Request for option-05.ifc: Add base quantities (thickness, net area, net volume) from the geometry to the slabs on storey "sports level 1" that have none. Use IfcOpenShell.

First a look at what the model holds.

```python
import ifcopenshell
import ifcopenshell.util.element
import ifcopenshell.util.unit

model = ifcopenshell.open("option-05.ifc")
print(model.schema)
for unit_type in ("LENGTHUNIT", "AREAUNIT", "VOLUMEUNIT"):
    print(unit_type, ifcopenshell.util.unit.calculate_unit_scale(model, unit_type))
storey = next(s for s in model.by_type("IfcBuildingStorey") if s.Name == "sports level 1")
slabs = [e for e in ifcopenshell.util.element.get_decomposition(storey) if e.is_a("IfcSlab")]
for e in sorted(slabs, key=lambda e: e.id()):
    print(e.id(), e.is_a(), e.Name, list(ifcopenshell.util.element.get_psets(e, qtos_only=True)), sep=" | ")
```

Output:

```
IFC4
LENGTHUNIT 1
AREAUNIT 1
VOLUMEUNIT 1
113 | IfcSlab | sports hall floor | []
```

```python
import ifcopenshell
import ifcopenshell.api.pset
import ifcopenshell.geom
import ifcopenshell.util.element
import ifcopenshell.util.shape
import ifcopenshell.util.unit

model = ifcopenshell.open("option-05.ifc")
unit_scale = ifcopenshell.util.unit.calculate_unit_scale(model)
area_scale = ifcopenshell.util.unit.calculate_unit_scale(model, "AREAUNIT")
volume_scale = ifcopenshell.util.unit.calculate_unit_scale(model, "VOLUMEUNIT")
settings = ifcopenshell.geom.settings()

storey = next(s for s in model.by_type("IfcBuildingStorey") if s.Name == "sports level 1")
slabs = [e for e in ifcopenshell.util.element.get_decomposition(storey) if e.is_a("IfcSlab")]

for e in sorted(slabs, key=lambda e: e.id()):
    if ifcopenshell.util.element.get_psets(e, qtos_only=True, should_inherit=False):
        continue
    # Geometry comes back in metres, in the element's own axes.
    shape = ifcopenshell.geom.create_shape(settings, e)
    values = {
        "Width": ifcopenshell.util.shape.get_z(shape.geometry) / unit_scale,
        "NetArea": ifcopenshell.util.shape.get_footprint_area(shape.geometry) / area_scale,
        "NetVolume": ifcopenshell.util.shape.get_volume(shape.geometry) / volume_scale,
    }
    qto = ifcopenshell.api.pset.add_qto(model, product=e, name="Qto_SlabBaseQuantities")
    ifcopenshell.api.pset.edit_qto(model, qto=qto, properties=values)
    print(e.id(), {k: round(v, 3) for k, v in values.items()})

model.write("option-05_v2.ifc")
```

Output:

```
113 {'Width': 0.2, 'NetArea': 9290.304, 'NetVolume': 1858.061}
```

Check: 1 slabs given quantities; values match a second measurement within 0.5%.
